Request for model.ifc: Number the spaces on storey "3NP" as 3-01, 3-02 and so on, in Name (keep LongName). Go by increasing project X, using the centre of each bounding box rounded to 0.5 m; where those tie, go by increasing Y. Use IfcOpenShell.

First a look at what the model holds.

```python
import ifcopenshell
import ifcopenshell.util.element
import ifcopenshell.util.placement

model = ifcopenshell.open("model.ifc")
print(model.schema)
storey = next(s for s in model.by_type("IfcBuildingStorey") if s.Name == "3NP")
spaces = [e for e in ifcopenshell.util.element.get_decomposition(storey) if e.is_a("IfcSpace")]
for e in sorted(spaces, key=lambda e: e.id()):
    origin = ifcopenshell.util.placement.get_local_placement(e.ObjectPlacement)[:3, 3]
    print(e.id(), e.Name, e.LongName, origin.round(2) + 0.0, sep=" | ")
```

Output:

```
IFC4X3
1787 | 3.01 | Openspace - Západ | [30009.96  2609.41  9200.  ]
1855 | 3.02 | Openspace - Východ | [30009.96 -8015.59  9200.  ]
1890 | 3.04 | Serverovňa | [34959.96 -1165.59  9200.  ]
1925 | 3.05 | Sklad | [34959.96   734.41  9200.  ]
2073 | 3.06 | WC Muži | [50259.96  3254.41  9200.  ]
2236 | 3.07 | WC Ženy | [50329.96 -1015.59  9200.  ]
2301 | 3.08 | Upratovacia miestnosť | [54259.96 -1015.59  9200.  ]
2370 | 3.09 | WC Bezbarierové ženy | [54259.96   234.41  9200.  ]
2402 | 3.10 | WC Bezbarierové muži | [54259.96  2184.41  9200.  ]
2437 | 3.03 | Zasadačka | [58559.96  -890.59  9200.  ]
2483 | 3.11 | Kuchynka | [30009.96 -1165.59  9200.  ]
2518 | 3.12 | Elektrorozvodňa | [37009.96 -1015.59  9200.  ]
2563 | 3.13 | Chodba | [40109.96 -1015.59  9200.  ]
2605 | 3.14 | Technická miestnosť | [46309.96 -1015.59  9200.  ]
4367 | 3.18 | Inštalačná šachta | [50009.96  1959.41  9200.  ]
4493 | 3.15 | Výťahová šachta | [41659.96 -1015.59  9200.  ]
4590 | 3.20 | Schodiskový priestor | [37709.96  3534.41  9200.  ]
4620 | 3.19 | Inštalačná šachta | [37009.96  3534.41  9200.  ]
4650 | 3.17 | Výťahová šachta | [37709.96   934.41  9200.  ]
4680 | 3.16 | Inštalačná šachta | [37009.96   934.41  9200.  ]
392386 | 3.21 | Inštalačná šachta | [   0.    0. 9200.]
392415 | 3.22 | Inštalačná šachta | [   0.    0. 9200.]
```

```python
import ifcopenshell
import ifcopenshell.geom
import ifcopenshell.util.element
import ifcopenshell.util.shape

model = ifcopenshell.open("model.ifc")
settings = ifcopenshell.geom.settings()
settings.set("use-world-coords", True)


def centre(element):
    shape = ifcopenshell.geom.create_shape(settings, element)
    return ifcopenshell.util.shape.get_bbox_centroid(shape.geometry)


storey = next(s for s in model.by_type("IfcBuildingStorey") if s.Name == "3NP")
spaces = [e for e in ifcopenshell.util.element.get_decomposition(storey) if e.is_a("IfcSpace")]

# Insertion points can sit at a corner or the storey origin, so sort by the geometry (in metres).
centres = {e: centre(e) for e in spaces}
spaces.sort(key=lambda e: (round(centres[e][0] / 0.5), centres[e][1]))

for i, e in enumerate(spaces, start=1):
    number = f"3-{i:02d}"
    e.Name = number
    print(e.id(), number)

model.write("model-out.ifc")
```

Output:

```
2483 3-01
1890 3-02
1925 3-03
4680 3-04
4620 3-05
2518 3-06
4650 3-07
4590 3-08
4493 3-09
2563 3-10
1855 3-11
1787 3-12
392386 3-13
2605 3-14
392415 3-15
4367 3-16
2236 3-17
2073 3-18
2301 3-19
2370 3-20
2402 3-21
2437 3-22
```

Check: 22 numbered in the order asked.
